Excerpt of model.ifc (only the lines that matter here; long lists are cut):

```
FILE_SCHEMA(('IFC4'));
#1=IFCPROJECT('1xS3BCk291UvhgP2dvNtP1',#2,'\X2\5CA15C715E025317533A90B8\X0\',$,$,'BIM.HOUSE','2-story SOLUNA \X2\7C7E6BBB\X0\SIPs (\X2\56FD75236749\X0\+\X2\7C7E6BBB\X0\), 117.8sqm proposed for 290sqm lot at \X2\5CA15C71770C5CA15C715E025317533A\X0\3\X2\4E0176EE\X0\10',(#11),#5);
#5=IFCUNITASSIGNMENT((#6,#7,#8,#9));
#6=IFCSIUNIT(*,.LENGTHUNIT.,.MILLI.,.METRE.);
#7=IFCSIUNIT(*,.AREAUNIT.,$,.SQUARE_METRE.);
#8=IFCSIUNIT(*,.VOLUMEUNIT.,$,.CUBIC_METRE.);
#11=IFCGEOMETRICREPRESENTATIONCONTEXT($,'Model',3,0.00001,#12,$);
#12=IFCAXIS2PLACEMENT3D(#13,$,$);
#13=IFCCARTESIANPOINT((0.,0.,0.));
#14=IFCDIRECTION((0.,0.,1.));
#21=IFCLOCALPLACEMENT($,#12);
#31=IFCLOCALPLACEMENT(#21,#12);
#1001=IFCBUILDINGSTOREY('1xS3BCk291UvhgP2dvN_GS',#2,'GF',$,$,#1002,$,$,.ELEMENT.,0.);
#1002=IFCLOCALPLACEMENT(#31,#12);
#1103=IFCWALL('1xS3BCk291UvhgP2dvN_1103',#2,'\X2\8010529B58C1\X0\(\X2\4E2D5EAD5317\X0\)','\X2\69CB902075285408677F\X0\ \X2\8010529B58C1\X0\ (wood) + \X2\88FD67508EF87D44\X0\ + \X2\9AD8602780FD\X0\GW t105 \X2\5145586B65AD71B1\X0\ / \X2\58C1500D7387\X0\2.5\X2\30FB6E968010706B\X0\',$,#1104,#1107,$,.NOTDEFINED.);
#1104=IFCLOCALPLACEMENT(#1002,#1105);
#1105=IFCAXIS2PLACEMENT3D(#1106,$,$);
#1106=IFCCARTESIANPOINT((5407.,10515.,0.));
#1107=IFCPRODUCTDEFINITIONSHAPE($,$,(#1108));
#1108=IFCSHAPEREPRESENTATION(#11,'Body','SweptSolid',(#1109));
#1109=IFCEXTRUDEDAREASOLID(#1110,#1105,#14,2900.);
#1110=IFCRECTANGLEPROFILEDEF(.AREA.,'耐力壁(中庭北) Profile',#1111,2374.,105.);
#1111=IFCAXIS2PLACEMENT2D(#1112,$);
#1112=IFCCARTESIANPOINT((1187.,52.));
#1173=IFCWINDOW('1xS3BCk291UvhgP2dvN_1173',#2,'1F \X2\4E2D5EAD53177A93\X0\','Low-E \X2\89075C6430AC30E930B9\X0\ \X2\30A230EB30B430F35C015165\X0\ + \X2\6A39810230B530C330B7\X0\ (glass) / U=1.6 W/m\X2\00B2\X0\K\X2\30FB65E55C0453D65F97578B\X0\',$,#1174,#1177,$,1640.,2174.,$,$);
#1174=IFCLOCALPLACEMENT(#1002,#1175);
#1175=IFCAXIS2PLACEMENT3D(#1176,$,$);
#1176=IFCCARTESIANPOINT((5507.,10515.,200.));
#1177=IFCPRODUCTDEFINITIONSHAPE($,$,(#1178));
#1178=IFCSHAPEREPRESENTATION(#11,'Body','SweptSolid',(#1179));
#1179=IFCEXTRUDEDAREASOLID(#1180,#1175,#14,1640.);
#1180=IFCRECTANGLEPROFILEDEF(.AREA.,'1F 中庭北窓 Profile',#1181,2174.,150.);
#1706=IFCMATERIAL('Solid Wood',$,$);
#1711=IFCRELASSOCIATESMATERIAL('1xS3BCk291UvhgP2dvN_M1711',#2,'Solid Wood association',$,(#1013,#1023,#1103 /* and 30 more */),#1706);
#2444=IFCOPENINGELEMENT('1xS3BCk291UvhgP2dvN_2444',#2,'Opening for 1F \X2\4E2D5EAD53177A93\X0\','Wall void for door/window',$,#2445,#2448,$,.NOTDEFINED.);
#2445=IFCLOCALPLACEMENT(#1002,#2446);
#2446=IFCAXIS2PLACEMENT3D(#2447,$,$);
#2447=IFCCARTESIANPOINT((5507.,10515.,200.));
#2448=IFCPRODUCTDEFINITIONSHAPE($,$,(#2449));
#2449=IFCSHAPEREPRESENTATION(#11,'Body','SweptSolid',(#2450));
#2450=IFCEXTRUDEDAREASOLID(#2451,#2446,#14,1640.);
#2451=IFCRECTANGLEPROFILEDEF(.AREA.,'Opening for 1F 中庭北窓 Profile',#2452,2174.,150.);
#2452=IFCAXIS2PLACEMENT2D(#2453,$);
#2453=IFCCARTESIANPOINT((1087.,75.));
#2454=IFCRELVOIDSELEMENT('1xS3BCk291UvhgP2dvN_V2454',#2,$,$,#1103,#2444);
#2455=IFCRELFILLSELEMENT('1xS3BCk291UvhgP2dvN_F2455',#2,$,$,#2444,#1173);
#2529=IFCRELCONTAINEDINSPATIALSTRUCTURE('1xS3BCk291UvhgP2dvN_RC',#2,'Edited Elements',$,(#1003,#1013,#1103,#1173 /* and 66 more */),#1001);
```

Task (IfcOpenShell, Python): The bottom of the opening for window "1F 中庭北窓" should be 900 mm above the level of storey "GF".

```python
import numpy as np
import ifcopenshell
import ifcopenshell.api.geometry
import ifcopenshell.geom
import ifcopenshell.util.element
import ifcopenshell.util.placement
import ifcopenshell.util.shape
import ifcopenshell.util.unit

model = ifcopenshell.open("model.ifc")
unit_scale = ifcopenshell.util.unit.calculate_unit_scale(model)

window = model.by_guid("1xS3BCk291UvhgP2dvN_1173")
opening = window.FillsVoids[0].RelatingOpeningElement
storey = ifcopenshell.util.element.get_container(window, ifc_class="IfcBuildingStorey")
level = ifcopenshell.util.placement.get_local_placement(storey.ObjectPlacement)[2, 3]

# The opening's origin need not be at the sill, so measure its lowest point.
shape = ifcopenshell.geom.create_shape(ifcopenshell.geom.settings(), opening)
bottom = ifcopenshell.util.shape.get_shape_bottom_elevation(shape, shape.geometry) / unit_scale
dz = level + 0.9 / unit_scale - bottom

shift = np.array([0.0, 0.0, dz])
# The window is not placed relative to its opening, so move both.
for product in (opening, window):
    matrix = ifcopenshell.util.placement.get_local_placement(product.ObjectPlacement)
    matrix[:3, 3] += shift
    ifcopenshell.api.geometry.edit_object_placement(model, product=product, matrix=matrix, is_si=False)

print(f"moved by {dz * unit_scale:+.3f} m")

model.write("model_updated.ifc")
```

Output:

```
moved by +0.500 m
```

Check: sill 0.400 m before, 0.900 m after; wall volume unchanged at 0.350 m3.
